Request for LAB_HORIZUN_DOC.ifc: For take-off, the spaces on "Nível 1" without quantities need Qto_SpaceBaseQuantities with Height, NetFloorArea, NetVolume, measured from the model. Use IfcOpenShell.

First a look at what the model holds.

```python
import ifcopenshell
import ifcopenshell.util.element
import ifcopenshell.util.unit

model = ifcopenshell.open("LAB_HORIZUN_DOC.ifc")
print(model.schema)
for unit_type in ("LENGTHUNIT", "AREAUNIT", "VOLUMEUNIT"):
    print(unit_type, ifcopenshell.util.unit.calculate_unit_scale(model, unit_type))
storey = next(s for s in model.by_type("IfcBuildingStorey") if s.Name == "Nível 1")
spaces = [e for e in ifcopenshell.util.element.get_decomposition(storey) if e.is_a("IfcSpace")]
for e in sorted(spaces, key=lambda e: e.id()):
    print(e.id(), e.is_a(), e.Name, list(ifcopenshell.util.element.get_psets(e, qtos_only=True)), sep=" | ")
```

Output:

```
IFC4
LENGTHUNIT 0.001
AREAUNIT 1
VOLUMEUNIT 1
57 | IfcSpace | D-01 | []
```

```python
import ifcopenshell
import ifcopenshell.api.pset
import ifcopenshell.geom
import ifcopenshell.util.element
import ifcopenshell.util.shape
import ifcopenshell.util.unit

model = ifcopenshell.open("LAB_HORIZUN_DOC.ifc")
unit_scale = ifcopenshell.util.unit.calculate_unit_scale(model)
area_scale = ifcopenshell.util.unit.calculate_unit_scale(model, "AREAUNIT")
volume_scale = ifcopenshell.util.unit.calculate_unit_scale(model, "VOLUMEUNIT")
settings = ifcopenshell.geom.settings()

storey = next(s for s in model.by_type("IfcBuildingStorey") if s.Name == "Nível 1")
spaces = [e for e in ifcopenshell.util.element.get_decomposition(storey) if e.is_a("IfcSpace")]

for e in sorted(spaces, key=lambda e: e.id()):
    if ifcopenshell.util.element.get_psets(e, qtos_only=True, should_inherit=False):
        continue
    # Geometry comes back in metres, in the element's own axes.
    shape = ifcopenshell.geom.create_shape(settings, e)
    values = {
        "Height": ifcopenshell.util.shape.get_z(shape.geometry) / unit_scale,
        "NetFloorArea": ifcopenshell.util.shape.get_footprint_area(shape.geometry) / area_scale,
        "NetVolume": ifcopenshell.util.shape.get_volume(shape.geometry) / volume_scale,
    }
    qto = ifcopenshell.api.pset.add_qto(model, product=e, name="Qto_SpaceBaseQuantities")
    ifcopenshell.api.pset.edit_qto(model, qto=qto, properties=values)
    print(e.id(), {k: round(v, 3) for k, v in values.items()})

model.write("LAB_HORIZUN_DOC-out.ifc")
```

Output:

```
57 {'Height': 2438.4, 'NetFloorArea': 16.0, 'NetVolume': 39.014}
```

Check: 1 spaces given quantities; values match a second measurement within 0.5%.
